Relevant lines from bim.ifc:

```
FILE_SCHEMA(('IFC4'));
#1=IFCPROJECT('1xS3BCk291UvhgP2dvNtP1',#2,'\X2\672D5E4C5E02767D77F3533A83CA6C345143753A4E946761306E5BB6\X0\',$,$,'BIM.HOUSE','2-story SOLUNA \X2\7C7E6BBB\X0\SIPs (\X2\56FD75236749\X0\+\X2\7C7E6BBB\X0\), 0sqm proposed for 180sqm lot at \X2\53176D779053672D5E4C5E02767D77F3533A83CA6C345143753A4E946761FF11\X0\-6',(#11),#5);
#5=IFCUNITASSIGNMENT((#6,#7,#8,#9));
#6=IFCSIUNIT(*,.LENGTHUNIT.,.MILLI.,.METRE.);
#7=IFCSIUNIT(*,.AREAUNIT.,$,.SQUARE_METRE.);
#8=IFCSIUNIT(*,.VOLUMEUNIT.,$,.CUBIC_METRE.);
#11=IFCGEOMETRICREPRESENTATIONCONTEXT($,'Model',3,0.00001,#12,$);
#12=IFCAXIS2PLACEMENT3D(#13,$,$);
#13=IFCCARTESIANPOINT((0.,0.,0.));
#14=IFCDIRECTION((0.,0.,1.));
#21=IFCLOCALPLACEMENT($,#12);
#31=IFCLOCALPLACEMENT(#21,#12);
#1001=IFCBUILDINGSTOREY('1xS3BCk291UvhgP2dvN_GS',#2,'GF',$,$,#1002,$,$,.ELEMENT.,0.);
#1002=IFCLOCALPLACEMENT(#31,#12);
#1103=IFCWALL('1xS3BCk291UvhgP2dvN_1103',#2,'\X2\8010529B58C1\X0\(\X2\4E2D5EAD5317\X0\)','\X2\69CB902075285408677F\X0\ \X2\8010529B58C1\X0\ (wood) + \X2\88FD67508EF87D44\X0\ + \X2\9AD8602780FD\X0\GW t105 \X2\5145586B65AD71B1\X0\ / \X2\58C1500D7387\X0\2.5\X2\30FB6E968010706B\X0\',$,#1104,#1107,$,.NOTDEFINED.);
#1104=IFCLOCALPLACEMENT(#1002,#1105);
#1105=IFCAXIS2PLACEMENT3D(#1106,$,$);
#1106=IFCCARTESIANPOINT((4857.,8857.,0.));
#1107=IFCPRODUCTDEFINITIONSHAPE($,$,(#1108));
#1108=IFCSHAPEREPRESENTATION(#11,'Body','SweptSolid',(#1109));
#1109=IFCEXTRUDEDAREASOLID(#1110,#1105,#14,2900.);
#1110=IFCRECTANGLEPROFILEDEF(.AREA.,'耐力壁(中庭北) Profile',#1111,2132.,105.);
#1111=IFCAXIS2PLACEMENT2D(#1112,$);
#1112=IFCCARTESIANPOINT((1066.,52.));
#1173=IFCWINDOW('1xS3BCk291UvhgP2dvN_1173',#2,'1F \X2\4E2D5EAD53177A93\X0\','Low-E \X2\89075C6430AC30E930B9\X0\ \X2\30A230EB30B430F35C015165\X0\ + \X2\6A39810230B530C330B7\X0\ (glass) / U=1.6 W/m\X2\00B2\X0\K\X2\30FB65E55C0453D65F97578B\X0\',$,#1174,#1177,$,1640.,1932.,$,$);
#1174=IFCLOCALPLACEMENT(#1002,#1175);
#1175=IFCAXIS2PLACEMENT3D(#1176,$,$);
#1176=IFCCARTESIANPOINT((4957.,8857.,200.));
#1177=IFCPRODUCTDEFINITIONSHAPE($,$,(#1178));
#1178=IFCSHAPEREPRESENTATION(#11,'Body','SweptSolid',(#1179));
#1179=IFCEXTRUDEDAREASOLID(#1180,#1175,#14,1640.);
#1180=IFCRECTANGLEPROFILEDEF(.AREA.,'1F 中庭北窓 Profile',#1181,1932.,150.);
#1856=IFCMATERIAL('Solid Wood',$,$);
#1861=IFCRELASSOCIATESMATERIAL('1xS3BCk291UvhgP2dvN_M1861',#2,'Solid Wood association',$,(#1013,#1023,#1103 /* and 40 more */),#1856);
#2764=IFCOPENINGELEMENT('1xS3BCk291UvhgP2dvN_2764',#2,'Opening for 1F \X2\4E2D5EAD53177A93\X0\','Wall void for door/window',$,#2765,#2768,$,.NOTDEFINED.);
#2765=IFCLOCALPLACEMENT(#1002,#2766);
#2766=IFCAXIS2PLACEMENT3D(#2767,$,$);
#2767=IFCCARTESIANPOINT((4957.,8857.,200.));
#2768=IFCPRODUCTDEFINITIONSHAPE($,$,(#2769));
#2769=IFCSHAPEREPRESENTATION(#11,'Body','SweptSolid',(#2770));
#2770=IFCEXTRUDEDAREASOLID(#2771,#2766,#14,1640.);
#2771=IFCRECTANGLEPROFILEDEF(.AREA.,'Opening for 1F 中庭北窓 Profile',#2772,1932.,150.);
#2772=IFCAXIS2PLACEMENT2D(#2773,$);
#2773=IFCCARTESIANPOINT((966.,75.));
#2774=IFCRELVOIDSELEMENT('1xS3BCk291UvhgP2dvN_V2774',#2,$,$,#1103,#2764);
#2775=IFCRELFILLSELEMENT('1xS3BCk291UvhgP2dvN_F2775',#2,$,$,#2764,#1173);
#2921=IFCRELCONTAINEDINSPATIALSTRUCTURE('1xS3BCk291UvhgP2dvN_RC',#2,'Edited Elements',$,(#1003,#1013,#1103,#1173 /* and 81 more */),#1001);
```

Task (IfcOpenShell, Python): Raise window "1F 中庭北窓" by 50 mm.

```python
import numpy as np
import ifcopenshell
import ifcopenshell.api.geometry
import ifcopenshell.util.placement
import ifcopenshell.util.unit

model = ifcopenshell.open("bim.ifc")
unit_scale = ifcopenshell.util.unit.calculate_unit_scale(model)

window = model.by_guid("1xS3BCk291UvhgP2dvN_1173")
opening = window.FillsVoids[0].RelatingOpeningElement
dz = 50.0

shift = np.array([0.0, 0.0, dz])
# The window is not placed relative to its opening, so move both.
for product in (opening, window):
    matrix = ifcopenshell.util.placement.get_local_placement(product.ObjectPlacement)
    matrix[:3, 3] += shift
    ifcopenshell.api.geometry.edit_object_placement(model, product=product, matrix=matrix, is_si=False)

print(f"moved by {dz * unit_scale:+.3f} m")

model.write("bim_rev.ifc")
```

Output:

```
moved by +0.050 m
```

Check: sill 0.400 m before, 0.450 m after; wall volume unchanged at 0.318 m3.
